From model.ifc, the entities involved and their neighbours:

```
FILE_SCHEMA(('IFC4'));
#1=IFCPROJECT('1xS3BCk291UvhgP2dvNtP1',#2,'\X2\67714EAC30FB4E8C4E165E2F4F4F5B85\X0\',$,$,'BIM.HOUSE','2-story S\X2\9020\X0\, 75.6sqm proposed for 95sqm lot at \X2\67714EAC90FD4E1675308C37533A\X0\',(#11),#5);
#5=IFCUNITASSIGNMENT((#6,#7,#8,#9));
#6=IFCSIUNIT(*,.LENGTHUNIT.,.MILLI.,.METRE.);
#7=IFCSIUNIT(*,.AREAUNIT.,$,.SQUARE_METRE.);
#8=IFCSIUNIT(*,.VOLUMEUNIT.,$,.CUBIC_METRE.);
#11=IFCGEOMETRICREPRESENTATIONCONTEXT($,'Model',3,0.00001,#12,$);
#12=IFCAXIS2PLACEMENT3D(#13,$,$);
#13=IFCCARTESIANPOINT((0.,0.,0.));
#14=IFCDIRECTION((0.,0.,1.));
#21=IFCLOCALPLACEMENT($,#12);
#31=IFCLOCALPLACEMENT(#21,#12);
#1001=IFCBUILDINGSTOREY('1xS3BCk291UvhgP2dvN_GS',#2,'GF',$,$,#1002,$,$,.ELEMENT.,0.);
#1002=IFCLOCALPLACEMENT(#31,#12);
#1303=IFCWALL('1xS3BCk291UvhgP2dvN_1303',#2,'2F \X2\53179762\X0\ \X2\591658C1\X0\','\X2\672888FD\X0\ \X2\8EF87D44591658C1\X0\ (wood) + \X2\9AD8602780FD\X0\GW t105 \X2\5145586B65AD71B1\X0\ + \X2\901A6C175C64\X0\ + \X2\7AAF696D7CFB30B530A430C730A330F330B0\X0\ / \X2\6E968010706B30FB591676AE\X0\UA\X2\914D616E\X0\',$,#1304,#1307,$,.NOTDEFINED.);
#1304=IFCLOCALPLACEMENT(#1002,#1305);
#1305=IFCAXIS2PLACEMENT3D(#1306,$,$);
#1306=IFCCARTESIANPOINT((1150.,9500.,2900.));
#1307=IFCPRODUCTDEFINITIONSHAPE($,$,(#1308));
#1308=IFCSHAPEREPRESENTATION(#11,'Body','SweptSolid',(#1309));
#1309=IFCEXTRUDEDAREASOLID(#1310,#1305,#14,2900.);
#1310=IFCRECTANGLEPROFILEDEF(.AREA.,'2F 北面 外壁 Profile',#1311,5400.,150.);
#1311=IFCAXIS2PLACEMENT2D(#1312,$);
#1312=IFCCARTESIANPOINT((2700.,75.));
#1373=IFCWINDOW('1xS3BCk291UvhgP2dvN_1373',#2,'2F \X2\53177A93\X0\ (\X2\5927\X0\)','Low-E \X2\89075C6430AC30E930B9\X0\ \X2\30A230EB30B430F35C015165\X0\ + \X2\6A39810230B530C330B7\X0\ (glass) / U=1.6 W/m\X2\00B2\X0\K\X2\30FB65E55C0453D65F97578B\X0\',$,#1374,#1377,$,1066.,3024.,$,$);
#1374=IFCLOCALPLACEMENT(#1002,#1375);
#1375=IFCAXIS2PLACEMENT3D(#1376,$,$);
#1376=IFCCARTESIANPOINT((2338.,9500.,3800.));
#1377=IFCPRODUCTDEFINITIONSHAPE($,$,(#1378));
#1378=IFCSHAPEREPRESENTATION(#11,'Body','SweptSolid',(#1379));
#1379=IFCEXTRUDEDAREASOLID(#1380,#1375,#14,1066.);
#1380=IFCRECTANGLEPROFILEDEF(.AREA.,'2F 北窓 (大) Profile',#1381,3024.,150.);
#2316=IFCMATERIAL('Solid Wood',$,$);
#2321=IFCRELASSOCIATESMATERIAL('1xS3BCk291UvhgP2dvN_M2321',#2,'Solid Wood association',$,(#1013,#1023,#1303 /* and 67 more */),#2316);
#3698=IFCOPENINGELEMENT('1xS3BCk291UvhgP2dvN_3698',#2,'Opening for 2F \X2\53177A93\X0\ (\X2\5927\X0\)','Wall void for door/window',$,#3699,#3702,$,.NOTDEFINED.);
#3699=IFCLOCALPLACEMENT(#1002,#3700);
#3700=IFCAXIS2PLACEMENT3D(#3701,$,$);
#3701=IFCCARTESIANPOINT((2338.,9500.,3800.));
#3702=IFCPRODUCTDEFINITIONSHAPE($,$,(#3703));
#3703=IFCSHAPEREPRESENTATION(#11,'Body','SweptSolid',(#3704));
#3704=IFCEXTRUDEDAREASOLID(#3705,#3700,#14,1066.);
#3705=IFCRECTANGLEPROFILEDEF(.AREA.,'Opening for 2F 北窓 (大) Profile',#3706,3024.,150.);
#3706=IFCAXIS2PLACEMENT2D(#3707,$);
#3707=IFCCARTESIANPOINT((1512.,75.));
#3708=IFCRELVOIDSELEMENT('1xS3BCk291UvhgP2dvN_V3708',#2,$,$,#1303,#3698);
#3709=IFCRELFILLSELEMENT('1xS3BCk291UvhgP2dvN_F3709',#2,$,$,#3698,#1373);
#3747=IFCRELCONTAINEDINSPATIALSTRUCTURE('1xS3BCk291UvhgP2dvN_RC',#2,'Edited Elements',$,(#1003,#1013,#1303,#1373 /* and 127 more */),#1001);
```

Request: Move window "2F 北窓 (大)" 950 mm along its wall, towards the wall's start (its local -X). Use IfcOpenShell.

```python
import ifcopenshell
import ifcopenshell.api.geometry
import ifcopenshell.util.placement
import ifcopenshell.util.unit

model = ifcopenshell.open("model.ifc")
unit_scale = ifcopenshell.util.unit.calculate_unit_scale(model)

window = model.by_guid("1xS3BCk291UvhgP2dvN_1373")
opening = window.FillsVoids[0].RelatingOpeningElement
wall = opening.VoidsElements[0].RelatingBuildingElement

wall_matrix = ifcopenshell.util.placement.get_local_placement(wall.ObjectPlacement)
shift = wall_matrix[:3, 0] * -0.95 / unit_scale
before = ifcopenshell.util.placement.get_local_placement(window.ObjectPlacement)[:3, 3].copy()

# The window is not placed relative to its opening, so move both.
for product in (opening, window):
    matrix = ifcopenshell.util.placement.get_local_placement(product.ObjectPlacement)
    matrix[:3, 3] += shift
    ifcopenshell.api.geometry.edit_object_placement(model, product=product, matrix=matrix, is_si=False)

after = ifcopenshell.util.placement.get_local_placement(window.ObjectPlacement)[:3, 3]
print("window moved by", (after - before).round(3) + 0.0)

model.write("model_updated.ifc")
```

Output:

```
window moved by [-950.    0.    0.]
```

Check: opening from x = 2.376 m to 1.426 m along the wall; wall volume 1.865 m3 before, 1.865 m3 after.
